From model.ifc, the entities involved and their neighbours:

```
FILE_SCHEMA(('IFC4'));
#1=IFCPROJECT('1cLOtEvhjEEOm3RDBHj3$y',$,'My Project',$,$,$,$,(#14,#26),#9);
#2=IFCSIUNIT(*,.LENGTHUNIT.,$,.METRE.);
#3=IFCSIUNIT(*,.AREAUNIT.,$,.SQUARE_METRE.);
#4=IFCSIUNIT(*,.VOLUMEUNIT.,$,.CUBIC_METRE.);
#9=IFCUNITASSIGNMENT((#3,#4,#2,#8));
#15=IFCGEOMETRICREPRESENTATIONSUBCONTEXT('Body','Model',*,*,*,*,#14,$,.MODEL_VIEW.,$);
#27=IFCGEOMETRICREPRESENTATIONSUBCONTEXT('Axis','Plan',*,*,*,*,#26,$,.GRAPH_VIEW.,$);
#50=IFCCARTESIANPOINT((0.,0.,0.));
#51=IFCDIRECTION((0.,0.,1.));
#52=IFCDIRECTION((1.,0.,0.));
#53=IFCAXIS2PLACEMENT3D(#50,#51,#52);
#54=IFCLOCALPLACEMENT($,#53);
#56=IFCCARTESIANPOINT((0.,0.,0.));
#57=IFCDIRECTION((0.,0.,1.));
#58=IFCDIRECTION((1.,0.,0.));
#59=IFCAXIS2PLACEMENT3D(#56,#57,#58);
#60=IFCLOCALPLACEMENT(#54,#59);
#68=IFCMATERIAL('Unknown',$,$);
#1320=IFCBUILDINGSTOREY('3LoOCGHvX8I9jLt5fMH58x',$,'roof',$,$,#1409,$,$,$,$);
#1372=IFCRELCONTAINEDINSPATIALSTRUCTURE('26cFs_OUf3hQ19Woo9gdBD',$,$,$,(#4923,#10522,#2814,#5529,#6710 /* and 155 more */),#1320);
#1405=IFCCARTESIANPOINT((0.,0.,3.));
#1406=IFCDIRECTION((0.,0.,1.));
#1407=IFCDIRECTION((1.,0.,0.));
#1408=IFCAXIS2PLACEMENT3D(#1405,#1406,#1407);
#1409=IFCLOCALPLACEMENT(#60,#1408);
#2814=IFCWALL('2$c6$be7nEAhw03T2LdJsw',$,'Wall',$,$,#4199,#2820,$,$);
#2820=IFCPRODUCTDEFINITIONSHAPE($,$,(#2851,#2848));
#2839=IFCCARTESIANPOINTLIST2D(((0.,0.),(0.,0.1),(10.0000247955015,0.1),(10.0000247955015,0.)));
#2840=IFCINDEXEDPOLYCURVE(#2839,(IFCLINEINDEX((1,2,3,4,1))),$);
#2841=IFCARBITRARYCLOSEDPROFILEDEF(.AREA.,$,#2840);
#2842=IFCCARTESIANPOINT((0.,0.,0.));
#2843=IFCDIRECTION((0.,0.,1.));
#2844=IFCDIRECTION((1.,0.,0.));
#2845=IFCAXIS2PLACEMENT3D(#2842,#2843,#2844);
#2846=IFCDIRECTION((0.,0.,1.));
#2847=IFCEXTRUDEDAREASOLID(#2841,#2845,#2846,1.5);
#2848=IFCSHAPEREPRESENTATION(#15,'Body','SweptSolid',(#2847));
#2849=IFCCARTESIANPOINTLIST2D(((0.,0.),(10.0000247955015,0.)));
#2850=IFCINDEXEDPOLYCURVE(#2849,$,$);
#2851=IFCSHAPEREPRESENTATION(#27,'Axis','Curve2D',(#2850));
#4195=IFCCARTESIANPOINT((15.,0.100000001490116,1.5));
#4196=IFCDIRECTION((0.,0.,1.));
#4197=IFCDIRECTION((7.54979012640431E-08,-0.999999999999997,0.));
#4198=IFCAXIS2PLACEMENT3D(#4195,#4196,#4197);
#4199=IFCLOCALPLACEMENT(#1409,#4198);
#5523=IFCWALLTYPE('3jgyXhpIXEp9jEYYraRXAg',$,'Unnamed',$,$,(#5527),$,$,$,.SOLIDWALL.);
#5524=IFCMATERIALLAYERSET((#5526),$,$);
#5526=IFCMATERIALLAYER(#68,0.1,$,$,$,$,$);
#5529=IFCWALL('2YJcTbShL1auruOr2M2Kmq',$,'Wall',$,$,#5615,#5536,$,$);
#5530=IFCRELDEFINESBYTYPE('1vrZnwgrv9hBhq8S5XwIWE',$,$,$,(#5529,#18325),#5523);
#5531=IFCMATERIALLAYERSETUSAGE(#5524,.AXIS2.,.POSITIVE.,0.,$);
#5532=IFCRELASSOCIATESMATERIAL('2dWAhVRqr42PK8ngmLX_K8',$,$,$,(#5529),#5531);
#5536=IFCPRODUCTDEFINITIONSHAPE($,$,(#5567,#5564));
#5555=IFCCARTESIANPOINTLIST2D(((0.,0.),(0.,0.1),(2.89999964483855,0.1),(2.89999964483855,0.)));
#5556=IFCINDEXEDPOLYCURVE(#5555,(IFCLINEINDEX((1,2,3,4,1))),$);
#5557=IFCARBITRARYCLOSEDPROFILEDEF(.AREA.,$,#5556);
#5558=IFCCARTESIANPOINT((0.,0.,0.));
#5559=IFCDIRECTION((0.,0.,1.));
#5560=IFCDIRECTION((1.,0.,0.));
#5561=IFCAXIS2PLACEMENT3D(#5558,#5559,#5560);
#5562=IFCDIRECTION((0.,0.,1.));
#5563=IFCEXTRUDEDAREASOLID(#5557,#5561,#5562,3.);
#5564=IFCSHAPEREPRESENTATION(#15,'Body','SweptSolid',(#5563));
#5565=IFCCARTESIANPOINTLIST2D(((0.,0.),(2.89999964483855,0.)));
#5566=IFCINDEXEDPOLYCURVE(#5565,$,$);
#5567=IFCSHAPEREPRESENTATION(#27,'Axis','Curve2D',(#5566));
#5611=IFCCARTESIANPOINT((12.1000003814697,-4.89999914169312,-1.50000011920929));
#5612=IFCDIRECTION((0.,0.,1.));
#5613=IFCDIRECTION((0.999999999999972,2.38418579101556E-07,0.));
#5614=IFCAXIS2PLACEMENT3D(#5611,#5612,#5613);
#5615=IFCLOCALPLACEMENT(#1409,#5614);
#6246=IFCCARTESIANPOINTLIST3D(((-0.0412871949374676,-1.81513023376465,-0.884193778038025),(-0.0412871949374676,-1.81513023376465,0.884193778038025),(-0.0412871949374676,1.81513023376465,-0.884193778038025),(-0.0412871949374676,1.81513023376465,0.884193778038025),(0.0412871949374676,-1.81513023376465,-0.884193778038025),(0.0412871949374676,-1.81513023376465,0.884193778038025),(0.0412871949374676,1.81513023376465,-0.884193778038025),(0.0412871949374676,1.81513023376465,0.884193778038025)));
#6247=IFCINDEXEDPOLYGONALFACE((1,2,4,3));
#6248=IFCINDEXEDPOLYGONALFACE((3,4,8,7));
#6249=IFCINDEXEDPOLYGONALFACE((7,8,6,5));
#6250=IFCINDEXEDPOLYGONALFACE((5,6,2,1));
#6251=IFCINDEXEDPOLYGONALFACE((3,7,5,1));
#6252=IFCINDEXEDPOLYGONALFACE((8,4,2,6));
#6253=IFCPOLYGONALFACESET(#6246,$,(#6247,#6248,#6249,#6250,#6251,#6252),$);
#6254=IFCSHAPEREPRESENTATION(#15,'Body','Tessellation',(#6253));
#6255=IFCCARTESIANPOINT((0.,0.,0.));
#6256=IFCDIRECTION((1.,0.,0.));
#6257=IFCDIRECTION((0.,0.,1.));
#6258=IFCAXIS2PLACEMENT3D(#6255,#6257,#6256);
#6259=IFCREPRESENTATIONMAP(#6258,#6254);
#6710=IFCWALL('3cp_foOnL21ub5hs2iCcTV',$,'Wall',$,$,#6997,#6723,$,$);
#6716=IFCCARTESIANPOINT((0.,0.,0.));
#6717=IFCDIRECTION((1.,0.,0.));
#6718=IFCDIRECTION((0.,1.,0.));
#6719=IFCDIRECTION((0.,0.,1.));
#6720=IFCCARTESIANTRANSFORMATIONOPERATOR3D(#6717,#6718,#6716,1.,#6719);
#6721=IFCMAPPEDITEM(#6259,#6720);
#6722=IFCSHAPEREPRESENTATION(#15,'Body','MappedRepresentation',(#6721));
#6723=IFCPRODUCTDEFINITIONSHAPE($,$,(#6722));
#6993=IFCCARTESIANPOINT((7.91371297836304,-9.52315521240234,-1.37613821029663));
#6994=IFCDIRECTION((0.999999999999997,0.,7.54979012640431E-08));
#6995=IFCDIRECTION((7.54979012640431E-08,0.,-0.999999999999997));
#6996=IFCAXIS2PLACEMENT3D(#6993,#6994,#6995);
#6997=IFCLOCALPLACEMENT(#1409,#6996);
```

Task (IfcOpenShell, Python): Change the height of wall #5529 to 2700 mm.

```python
import ifcopenshell
import ifcopenshell.geom
import ifcopenshell.util.representation
import ifcopenshell.util.shape

model = ifcopenshell.open("model.ifc")
settings = ifcopenshell.geom.settings()


def volume(element):
    """Net volume in cubic metres, openings subtracted."""
    shape = ifcopenshell.geom.create_shape(settings, element)
    return ifcopenshell.util.shape.get_volume(shape.geometry)


wall = model.by_id(5529)
before = volume(wall)

body = ifcopenshell.util.representation.get_representation(wall, "Model", "Body")
solid = body.Items[0]
old_height = solid.Depth
solid.Depth = 2.7
after = volume(wall)

print(f"height {old_height:g} -> {solid.Depth:g}, volume {before:.3f} -> {after:.3f} m3")

model.write("model-out.ifc")
```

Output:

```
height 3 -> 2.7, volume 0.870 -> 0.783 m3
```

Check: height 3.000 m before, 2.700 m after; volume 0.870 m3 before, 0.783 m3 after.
